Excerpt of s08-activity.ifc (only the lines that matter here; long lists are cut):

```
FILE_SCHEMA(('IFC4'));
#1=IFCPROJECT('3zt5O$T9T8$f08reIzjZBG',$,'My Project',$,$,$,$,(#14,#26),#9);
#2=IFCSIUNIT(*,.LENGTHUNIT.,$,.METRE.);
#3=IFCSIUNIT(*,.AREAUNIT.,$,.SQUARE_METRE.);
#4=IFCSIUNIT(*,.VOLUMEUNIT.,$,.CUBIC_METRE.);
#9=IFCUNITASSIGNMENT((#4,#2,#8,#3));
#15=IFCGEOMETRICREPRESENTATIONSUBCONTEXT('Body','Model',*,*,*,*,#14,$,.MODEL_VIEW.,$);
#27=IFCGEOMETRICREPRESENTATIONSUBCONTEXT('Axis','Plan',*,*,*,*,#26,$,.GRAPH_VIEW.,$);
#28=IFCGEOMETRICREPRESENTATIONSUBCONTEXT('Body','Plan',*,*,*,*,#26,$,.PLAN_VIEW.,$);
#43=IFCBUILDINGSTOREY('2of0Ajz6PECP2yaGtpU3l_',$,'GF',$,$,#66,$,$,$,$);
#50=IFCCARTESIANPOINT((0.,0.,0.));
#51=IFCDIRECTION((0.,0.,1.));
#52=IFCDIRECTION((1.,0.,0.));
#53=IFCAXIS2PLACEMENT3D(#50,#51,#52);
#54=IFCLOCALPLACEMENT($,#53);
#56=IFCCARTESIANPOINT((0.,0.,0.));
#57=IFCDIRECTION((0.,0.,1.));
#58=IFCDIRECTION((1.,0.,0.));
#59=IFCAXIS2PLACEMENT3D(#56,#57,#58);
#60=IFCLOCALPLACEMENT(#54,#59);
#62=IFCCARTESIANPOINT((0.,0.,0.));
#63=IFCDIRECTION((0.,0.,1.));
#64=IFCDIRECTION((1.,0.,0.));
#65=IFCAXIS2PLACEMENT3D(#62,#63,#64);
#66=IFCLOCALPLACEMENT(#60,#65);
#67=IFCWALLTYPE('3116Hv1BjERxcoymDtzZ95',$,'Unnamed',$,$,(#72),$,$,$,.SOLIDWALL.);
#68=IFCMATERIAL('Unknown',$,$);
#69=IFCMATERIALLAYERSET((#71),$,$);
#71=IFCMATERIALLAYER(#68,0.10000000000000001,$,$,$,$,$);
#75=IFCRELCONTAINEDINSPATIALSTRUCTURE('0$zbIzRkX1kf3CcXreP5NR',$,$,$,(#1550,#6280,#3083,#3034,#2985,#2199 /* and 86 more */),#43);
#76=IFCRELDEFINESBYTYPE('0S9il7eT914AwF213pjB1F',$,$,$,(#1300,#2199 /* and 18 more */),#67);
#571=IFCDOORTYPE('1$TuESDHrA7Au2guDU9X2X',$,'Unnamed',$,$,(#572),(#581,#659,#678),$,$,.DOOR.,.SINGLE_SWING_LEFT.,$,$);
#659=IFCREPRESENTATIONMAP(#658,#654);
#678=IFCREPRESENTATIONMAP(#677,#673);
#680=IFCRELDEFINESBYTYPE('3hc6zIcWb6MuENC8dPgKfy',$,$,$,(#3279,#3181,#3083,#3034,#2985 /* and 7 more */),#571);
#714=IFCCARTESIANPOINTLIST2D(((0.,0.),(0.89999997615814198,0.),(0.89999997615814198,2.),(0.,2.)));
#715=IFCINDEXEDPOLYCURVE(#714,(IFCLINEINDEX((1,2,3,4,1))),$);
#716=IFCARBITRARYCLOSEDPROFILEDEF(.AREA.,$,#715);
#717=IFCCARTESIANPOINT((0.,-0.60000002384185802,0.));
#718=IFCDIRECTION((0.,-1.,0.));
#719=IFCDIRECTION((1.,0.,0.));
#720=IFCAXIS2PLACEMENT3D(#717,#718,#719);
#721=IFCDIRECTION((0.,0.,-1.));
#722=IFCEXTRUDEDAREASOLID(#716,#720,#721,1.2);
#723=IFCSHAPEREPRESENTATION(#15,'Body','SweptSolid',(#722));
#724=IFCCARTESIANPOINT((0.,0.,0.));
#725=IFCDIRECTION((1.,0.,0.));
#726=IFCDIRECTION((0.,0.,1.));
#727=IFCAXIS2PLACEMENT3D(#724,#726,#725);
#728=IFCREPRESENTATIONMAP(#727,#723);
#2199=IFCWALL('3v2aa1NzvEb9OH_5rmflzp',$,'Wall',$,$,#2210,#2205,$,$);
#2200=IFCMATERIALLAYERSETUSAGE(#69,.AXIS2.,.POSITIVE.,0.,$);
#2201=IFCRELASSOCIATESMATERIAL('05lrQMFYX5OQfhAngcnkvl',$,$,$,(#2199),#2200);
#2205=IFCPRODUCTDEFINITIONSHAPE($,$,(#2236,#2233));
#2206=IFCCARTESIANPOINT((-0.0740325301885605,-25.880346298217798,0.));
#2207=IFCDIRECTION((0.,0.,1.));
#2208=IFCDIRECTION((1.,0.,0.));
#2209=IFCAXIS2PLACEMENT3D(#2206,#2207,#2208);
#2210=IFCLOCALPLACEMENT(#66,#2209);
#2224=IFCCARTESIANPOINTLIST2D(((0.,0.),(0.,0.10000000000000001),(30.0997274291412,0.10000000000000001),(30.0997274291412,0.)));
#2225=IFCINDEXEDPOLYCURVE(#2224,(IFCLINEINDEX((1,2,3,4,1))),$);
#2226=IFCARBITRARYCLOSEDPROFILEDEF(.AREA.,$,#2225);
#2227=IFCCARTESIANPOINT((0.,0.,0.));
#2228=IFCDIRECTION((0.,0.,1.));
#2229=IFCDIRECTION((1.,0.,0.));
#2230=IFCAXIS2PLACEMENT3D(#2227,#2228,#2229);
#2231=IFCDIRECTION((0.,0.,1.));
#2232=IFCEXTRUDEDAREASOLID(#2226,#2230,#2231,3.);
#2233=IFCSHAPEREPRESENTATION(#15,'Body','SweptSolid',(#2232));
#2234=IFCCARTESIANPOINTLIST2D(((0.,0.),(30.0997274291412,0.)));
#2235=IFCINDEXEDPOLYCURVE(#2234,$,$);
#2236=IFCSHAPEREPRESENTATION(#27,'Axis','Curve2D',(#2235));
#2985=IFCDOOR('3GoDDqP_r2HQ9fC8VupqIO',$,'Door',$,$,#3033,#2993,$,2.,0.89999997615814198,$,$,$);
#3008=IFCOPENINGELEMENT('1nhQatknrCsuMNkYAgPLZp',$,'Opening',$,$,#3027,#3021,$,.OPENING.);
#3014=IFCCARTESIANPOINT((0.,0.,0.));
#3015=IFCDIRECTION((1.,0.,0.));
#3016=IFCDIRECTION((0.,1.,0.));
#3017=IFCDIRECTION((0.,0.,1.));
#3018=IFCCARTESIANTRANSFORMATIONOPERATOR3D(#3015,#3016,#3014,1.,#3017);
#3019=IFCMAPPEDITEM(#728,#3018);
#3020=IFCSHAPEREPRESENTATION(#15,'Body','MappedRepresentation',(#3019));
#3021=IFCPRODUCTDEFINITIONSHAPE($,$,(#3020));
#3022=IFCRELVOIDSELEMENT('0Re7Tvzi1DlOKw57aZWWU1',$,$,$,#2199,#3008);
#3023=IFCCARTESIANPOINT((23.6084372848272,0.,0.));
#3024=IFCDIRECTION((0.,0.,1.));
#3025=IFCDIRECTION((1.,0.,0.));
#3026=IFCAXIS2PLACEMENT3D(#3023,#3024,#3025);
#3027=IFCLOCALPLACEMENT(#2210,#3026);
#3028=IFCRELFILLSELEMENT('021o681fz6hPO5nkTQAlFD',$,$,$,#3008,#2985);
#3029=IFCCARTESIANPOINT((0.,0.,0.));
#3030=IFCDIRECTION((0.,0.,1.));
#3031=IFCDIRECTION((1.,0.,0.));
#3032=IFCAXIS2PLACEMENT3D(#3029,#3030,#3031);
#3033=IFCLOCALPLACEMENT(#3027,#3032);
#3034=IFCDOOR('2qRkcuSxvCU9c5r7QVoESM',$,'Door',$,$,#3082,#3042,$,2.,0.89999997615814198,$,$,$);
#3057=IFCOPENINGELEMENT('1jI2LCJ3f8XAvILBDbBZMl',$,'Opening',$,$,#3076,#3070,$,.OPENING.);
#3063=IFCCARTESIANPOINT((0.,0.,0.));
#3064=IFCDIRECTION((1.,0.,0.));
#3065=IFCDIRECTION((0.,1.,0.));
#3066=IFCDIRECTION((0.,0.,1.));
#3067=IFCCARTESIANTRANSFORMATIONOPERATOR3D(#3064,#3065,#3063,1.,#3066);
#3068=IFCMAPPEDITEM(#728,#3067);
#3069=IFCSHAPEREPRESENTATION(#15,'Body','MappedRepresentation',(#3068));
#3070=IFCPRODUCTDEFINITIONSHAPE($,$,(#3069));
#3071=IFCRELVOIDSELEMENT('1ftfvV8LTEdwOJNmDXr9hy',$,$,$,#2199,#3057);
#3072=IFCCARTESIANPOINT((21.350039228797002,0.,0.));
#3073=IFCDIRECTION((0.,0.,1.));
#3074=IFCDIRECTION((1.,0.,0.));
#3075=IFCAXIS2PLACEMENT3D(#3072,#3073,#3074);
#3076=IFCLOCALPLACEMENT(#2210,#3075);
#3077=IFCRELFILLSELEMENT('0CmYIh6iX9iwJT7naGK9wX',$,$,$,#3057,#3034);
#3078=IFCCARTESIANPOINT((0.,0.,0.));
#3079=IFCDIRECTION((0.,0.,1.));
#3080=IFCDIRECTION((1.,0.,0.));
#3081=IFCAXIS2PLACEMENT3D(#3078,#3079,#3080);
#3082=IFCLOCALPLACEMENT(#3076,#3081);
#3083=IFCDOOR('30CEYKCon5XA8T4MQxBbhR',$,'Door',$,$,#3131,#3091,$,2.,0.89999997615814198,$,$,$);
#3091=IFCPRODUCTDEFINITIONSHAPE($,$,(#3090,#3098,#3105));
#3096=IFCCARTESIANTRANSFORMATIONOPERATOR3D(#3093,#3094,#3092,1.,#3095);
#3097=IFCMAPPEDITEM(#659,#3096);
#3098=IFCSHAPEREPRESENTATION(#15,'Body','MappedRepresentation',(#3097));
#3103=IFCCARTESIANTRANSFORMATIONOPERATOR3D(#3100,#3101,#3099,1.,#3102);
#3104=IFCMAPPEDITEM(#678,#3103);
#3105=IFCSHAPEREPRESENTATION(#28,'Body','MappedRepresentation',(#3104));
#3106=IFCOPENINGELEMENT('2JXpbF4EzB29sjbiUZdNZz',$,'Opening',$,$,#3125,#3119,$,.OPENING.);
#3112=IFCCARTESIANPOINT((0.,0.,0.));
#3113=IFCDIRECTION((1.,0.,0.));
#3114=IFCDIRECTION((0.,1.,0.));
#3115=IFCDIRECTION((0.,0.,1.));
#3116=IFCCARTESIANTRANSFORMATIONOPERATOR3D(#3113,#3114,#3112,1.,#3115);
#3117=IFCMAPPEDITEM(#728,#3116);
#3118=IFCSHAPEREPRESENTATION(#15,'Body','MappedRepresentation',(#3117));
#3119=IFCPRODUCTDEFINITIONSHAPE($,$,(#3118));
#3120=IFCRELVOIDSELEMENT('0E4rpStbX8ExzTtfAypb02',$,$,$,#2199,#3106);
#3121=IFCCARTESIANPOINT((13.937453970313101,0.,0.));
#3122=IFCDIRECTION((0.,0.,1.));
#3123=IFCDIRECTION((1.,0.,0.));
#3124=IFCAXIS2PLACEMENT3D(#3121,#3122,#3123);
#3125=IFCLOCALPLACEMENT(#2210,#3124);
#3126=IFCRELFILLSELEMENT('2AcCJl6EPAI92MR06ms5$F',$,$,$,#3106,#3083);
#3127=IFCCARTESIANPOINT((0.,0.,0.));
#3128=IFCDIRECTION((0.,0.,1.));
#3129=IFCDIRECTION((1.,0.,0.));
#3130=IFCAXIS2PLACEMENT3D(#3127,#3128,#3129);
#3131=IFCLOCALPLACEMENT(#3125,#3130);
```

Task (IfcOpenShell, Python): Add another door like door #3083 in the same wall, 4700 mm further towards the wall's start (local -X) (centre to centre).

```python
import ifcopenshell
import ifcopenshell.api.feature
import ifcopenshell.api.geometry
import ifcopenshell.api.root
import ifcopenshell.geom
import ifcopenshell.util.element
import ifcopenshell.util.placement
import ifcopenshell.util.shape

model = ifcopenshell.open("s08-activity.ifc")
settings = ifcopenshell.geom.settings()


def volume(element):
    """Net volume in cubic metres, openings subtracted."""
    shape = ifcopenshell.geom.create_shape(settings, element)
    return ifcopenshell.util.shape.get_volume(shape.geometry)


door = model.by_guid("30CEYKCon5XA8T4MQxBbhR")
opening = door.FillsVoids[0].RelatingOpeningElement
wall = opening.VoidsElements[0].RelatingBuildingElement
before = volume(wall)
shift = ifcopenshell.util.placement.get_local_placement(wall.ObjectPlacement)[:3, 0] * -4.7

# copy_class copies the void relationship, type, container and properties, but no geometry.
new_opening = ifcopenshell.api.root.copy_class(model, product=opening)
new_opening.Representation = ifcopenshell.util.element.copy_deep(
    model, opening.Representation, exclude=["IfcGeometricRepresentationContext", "IfcRepresentationMap"]
)
new_door = ifcopenshell.api.root.copy_class(model, product=door)
new_door.Representation = ifcopenshell.util.element.copy_deep(
    model, door.Representation, exclude=["IfcGeometricRepresentationContext", "IfcRepresentationMap"]
)
ifcopenshell.api.feature.add_filling(model, opening=new_opening, element=new_door)

for old, new in ((opening, new_opening), (door, new_door)):
    matrix = ifcopenshell.util.placement.get_local_placement(old.ObjectPlacement)
    matrix[:3, 3] += shift
    ifcopenshell.api.geometry.edit_object_placement(model, product=new, matrix=matrix, is_si=False)

after = volume(wall)

print(f"wall volume {before:.3f} -> {after:.3f} m3")

model.write("s08-activity-out.ifc")
```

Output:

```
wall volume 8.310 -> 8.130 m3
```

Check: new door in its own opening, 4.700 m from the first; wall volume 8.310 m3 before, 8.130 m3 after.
